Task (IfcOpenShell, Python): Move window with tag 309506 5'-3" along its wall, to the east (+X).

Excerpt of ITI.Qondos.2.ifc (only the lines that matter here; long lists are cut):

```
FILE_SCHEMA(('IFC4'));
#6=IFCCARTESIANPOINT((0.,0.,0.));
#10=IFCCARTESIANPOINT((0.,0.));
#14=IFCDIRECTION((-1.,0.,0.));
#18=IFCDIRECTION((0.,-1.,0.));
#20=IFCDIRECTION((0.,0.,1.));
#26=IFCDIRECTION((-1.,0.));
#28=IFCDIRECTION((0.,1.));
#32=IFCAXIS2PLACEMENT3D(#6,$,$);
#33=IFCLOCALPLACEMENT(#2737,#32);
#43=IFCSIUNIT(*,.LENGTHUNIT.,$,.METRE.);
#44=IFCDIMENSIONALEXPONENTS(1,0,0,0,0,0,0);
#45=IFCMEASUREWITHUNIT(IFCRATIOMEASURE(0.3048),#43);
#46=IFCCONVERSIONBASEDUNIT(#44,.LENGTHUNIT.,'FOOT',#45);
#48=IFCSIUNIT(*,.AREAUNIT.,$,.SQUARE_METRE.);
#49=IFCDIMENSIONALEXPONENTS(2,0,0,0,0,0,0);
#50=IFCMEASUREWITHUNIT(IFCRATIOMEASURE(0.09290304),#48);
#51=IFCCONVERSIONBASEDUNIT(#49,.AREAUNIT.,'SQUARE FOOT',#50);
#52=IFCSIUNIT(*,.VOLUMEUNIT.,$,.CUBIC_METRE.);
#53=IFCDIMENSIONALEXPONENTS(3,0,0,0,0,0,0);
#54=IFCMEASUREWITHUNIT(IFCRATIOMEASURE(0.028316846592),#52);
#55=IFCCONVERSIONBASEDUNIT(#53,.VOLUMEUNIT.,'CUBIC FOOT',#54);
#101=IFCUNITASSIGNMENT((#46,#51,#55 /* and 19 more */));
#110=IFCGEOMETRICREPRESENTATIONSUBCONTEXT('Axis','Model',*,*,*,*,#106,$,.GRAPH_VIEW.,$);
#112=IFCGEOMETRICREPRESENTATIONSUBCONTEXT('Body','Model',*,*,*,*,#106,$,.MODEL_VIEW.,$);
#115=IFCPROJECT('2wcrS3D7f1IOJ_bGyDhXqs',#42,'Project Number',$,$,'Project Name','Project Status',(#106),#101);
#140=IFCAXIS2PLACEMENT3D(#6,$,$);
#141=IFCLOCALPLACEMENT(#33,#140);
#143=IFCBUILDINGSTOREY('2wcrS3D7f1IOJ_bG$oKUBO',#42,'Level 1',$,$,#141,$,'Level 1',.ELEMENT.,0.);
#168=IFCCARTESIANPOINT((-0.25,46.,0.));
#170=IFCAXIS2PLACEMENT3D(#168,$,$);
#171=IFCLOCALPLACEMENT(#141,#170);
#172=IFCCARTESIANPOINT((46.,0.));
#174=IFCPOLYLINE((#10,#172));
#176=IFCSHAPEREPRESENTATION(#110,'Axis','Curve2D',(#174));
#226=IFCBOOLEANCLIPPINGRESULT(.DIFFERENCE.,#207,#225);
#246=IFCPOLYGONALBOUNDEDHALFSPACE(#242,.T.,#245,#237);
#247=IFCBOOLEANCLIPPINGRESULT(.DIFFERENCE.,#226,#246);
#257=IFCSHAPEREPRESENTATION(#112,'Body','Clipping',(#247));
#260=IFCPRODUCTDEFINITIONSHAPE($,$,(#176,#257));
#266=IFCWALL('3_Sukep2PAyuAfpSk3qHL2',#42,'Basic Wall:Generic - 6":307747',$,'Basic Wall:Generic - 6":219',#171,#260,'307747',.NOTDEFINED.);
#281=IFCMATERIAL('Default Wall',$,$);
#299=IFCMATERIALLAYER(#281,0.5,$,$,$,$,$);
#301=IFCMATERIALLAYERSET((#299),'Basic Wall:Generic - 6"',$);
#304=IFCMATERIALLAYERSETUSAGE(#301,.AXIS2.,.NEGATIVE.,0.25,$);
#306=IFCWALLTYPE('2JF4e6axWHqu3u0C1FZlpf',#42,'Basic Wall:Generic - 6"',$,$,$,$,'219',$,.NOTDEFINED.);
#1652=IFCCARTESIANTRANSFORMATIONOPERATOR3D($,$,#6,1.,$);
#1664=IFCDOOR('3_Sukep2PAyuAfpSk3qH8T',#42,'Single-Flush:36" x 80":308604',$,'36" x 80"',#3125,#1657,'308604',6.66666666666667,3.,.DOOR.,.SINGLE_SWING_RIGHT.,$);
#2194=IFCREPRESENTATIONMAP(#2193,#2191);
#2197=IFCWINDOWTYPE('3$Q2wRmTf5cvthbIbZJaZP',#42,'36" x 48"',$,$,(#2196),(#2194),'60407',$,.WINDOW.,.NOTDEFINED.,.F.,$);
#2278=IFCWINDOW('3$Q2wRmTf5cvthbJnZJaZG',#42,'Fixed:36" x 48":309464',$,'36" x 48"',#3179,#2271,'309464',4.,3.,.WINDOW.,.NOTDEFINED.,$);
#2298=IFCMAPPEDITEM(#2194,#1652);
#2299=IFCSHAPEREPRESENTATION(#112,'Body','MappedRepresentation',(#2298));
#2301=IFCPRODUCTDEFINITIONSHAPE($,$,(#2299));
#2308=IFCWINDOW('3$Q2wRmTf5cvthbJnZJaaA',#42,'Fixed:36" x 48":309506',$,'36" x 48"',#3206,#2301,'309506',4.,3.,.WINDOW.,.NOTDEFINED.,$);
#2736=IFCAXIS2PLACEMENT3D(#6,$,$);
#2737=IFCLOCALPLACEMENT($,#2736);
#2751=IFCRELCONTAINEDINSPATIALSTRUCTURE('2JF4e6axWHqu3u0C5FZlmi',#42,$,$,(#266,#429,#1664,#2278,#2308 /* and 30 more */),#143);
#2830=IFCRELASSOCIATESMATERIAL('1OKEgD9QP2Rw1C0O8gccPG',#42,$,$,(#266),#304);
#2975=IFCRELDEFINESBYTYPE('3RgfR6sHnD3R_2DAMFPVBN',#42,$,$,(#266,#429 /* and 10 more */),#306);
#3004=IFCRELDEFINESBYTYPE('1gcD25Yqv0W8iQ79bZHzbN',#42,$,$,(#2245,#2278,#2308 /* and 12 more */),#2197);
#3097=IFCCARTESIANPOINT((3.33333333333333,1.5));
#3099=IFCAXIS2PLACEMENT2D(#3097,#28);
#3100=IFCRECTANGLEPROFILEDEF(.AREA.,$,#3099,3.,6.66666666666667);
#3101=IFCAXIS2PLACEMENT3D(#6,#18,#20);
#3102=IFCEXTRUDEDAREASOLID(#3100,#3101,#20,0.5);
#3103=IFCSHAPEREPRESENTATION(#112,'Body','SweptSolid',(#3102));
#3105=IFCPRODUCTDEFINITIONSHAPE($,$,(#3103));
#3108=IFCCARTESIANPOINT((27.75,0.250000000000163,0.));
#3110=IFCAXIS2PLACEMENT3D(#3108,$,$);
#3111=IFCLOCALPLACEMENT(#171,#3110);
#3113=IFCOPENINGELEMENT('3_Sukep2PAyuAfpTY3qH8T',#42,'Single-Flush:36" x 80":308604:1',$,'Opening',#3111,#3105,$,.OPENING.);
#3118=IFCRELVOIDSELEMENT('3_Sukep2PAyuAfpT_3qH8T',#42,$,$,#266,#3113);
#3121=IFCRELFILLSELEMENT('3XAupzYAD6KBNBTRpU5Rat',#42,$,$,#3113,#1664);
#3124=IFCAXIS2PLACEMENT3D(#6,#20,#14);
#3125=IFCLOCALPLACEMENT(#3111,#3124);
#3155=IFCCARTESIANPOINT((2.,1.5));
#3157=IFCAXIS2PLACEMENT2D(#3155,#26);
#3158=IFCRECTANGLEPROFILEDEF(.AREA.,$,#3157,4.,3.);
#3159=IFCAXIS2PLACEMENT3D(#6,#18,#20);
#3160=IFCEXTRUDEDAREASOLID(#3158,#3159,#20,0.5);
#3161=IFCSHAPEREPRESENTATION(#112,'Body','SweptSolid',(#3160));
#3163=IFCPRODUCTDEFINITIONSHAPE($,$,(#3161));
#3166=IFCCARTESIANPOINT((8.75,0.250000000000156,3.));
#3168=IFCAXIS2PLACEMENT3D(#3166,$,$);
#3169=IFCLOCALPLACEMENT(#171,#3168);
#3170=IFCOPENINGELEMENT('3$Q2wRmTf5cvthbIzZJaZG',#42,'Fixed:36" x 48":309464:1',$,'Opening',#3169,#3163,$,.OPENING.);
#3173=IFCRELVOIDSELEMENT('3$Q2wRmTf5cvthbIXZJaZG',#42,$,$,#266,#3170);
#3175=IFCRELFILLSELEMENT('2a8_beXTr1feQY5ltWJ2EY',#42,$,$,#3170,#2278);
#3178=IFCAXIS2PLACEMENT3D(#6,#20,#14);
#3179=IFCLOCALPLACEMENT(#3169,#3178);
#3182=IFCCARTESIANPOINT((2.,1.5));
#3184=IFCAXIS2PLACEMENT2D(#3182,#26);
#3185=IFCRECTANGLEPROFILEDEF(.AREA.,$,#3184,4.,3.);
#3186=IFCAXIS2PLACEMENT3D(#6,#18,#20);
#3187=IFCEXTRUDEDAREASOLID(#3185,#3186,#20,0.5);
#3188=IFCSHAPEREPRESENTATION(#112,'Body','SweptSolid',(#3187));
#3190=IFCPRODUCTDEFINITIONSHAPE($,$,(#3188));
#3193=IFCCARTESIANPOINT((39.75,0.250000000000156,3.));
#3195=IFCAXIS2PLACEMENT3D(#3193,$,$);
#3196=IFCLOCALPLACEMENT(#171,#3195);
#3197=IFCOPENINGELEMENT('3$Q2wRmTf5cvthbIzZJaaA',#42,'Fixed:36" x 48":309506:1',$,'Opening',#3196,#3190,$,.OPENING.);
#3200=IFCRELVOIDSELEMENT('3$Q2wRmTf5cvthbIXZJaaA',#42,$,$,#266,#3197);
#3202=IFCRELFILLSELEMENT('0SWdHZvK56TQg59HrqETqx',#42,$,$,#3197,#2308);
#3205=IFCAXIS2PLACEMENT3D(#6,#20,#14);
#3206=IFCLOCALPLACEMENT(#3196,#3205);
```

```python
import ifcopenshell
import ifcopenshell.api.geometry
import ifcopenshell.util.placement
import ifcopenshell.util.unit

model = ifcopenshell.open("ITI.Qondos.2.ifc")
unit_scale = ifcopenshell.util.unit.calculate_unit_scale(model)

window = model.by_id(2308)
opening = window.FillsVoids[0].RelatingOpeningElement
wall = opening.VoidsElements[0].RelatingBuildingElement

wall_matrix = ifcopenshell.util.placement.get_local_placement(wall.ObjectPlacement)
shift = wall_matrix[:3, 0] * 63 * 0.0254 / unit_scale
before = ifcopenshell.util.placement.get_local_placement(window.ObjectPlacement)[:3, 3].copy()

# The window is placed relative to its opening, so it follows when the opening moves.
matrix = ifcopenshell.util.placement.get_local_placement(opening.ObjectPlacement)
matrix[:3, 3] += shift
ifcopenshell.api.geometry.edit_object_placement(
    model, product=opening, matrix=matrix, is_si=False, should_transform_children=True
)

after = ifcopenshell.util.placement.get_local_placement(window.ObjectPlacement)[:3, 3]
print("window moved by", (after - before).round(3) + 0.0)

model.write("ITI.Qondos.2-out.ifc")
```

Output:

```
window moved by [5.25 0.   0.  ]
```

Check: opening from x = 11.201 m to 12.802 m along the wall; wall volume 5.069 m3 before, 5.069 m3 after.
